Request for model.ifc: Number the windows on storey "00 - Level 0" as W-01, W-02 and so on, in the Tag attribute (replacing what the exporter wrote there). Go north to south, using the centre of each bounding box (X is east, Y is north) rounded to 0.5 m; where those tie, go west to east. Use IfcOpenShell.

First a look at what the model holds.

```python
import ifcopenshell
import ifcopenshell.util.element
import ifcopenshell.util.placement

model = ifcopenshell.open("model.ifc")
print(model.schema)
storey = next(s for s in model.by_type("IfcBuildingStorey") if s.Name == "00 - Level 0")
windows = [e for e in ifcopenshell.util.element.get_decomposition(storey) if e.is_a("IfcWindow")]
for e in sorted(windows, key=lambda e: e.id()):
    origin = ifcopenshell.util.placement.get_local_placement(e.ObjectPlacement)[:3, 3]
    print(e.id(), e.Tag, e.Name, origin.round(2) + 0.0, sep=" | ")
```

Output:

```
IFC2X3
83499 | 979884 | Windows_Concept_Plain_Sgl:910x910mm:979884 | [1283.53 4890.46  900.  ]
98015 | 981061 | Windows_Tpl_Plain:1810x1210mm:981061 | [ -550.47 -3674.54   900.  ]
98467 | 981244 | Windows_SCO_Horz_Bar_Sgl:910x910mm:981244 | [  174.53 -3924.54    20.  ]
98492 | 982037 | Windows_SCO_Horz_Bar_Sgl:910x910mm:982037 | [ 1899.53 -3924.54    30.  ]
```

```python
import ifcopenshell
import ifcopenshell.geom
import ifcopenshell.util.element
import ifcopenshell.util.shape

model = ifcopenshell.open("model.ifc")
settings = ifcopenshell.geom.settings()
settings.set("use-world-coords", True)


def centre(element):
    shape = ifcopenshell.geom.create_shape(settings, element)
    return ifcopenshell.util.shape.get_bbox_centroid(shape.geometry)


storey = next(s for s in model.by_type("IfcBuildingStorey") if s.Name == "00 - Level 0")
windows = [e for e in ifcopenshell.util.element.get_decomposition(storey) if e.is_a("IfcWindow")]

# Insertion points can sit at a corner or the storey origin, so sort by the geometry (in metres).
centres = {e: centre(e) for e in windows}
windows.sort(key=lambda e: (-round(centres[e][1] / 0.5), centres[e][0]))

for i, e in enumerate(windows, start=1):
    number = f"W-{i:02d}"
    e.Tag = number
    print(e.id(), number)

model.write("model_v2.ifc")
```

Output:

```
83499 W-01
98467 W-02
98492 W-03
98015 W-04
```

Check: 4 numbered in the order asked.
